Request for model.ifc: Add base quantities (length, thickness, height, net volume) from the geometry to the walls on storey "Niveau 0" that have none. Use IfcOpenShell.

First a look at what the model holds.

```python
import ifcopenshell
import ifcopenshell.util.element
import ifcopenshell.util.unit

model = ifcopenshell.open("model.ifc")
print(model.schema)
for unit_type in ("LENGTHUNIT", "AREAUNIT", "VOLUMEUNIT"):
    print(unit_type, ifcopenshell.util.unit.calculate_unit_scale(model, unit_type))
storey = next(s for s in model.by_type("IfcBuildingStorey") if s.Name == "Niveau 0")
walls = [e for e in ifcopenshell.util.element.get_decomposition(storey) if e.is_a("IfcWall")]
for e in sorted(walls, key=lambda e: e.id()):
    print(e.id(), e.is_a(), e.Name, list(ifcopenshell.util.element.get_psets(e, qtos_only=True)), sep=" | ")
```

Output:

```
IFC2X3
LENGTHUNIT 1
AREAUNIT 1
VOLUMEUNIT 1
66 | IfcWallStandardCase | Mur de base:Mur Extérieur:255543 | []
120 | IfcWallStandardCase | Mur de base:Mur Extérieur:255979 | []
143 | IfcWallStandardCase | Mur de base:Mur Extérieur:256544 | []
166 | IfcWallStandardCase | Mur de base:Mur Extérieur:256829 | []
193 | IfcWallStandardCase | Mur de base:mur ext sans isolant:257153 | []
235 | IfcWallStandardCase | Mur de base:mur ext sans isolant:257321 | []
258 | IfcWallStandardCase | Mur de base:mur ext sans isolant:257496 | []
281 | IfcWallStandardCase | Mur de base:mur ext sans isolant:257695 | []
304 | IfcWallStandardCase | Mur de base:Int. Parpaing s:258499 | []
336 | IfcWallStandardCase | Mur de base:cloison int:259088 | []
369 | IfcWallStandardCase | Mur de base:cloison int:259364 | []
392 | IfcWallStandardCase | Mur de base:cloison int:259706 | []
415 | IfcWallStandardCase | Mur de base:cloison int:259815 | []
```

```python
import ifcopenshell
import ifcopenshell.api.pset
import ifcopenshell.geom
import ifcopenshell.util.element
import ifcopenshell.util.shape
import ifcopenshell.util.unit

model = ifcopenshell.open("model.ifc")
unit_scale = ifcopenshell.util.unit.calculate_unit_scale(model)
volume_scale = ifcopenshell.util.unit.calculate_unit_scale(model, "VOLUMEUNIT")
settings = ifcopenshell.geom.settings()

storey = next(s for s in model.by_type("IfcBuildingStorey") if s.Name == "Niveau 0")
walls = [e for e in ifcopenshell.util.element.get_decomposition(storey) if e.is_a("IfcWall")]

for e in sorted(walls, key=lambda e: e.id()):
    if ifcopenshell.util.element.get_psets(e, qtos_only=True, should_inherit=False):
        continue
    # Geometry comes back in metres, in the element's own axes.
    shape = ifcopenshell.geom.create_shape(settings, e)
    values = {
        "Length": ifcopenshell.util.shape.get_x(shape.geometry) / unit_scale,
        "Width": ifcopenshell.util.shape.get_y(shape.geometry) / unit_scale,
        "Height": ifcopenshell.util.shape.get_z(shape.geometry) / unit_scale,
        "NetVolume": ifcopenshell.util.shape.get_volume(shape.geometry) / volume_scale,
    }
    qto = ifcopenshell.api.pset.add_qto(model, product=e, name="BaseQuantities")
    ifcopenshell.api.pset.edit_qto(model, qto=qto, properties=values)
    print(e.id(), {k: round(v, 3) for k, v in values.items()})

model.write("model_v2.ifc")
```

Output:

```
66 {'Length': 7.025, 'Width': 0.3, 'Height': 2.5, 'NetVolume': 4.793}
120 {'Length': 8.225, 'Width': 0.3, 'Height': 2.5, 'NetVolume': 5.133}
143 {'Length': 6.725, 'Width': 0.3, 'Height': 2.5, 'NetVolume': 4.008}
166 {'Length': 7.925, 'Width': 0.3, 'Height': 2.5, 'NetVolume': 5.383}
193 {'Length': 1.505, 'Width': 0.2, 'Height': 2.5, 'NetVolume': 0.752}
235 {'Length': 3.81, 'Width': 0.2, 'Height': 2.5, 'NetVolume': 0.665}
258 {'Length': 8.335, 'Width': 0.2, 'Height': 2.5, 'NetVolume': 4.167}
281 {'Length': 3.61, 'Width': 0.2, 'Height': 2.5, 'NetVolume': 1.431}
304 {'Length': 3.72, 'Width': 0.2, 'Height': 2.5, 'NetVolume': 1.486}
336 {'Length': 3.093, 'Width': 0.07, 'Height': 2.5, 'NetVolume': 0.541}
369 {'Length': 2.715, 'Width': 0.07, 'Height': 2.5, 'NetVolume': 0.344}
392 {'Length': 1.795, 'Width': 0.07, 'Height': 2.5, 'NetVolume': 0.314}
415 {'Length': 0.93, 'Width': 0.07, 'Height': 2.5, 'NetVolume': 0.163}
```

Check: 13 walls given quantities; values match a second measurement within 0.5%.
